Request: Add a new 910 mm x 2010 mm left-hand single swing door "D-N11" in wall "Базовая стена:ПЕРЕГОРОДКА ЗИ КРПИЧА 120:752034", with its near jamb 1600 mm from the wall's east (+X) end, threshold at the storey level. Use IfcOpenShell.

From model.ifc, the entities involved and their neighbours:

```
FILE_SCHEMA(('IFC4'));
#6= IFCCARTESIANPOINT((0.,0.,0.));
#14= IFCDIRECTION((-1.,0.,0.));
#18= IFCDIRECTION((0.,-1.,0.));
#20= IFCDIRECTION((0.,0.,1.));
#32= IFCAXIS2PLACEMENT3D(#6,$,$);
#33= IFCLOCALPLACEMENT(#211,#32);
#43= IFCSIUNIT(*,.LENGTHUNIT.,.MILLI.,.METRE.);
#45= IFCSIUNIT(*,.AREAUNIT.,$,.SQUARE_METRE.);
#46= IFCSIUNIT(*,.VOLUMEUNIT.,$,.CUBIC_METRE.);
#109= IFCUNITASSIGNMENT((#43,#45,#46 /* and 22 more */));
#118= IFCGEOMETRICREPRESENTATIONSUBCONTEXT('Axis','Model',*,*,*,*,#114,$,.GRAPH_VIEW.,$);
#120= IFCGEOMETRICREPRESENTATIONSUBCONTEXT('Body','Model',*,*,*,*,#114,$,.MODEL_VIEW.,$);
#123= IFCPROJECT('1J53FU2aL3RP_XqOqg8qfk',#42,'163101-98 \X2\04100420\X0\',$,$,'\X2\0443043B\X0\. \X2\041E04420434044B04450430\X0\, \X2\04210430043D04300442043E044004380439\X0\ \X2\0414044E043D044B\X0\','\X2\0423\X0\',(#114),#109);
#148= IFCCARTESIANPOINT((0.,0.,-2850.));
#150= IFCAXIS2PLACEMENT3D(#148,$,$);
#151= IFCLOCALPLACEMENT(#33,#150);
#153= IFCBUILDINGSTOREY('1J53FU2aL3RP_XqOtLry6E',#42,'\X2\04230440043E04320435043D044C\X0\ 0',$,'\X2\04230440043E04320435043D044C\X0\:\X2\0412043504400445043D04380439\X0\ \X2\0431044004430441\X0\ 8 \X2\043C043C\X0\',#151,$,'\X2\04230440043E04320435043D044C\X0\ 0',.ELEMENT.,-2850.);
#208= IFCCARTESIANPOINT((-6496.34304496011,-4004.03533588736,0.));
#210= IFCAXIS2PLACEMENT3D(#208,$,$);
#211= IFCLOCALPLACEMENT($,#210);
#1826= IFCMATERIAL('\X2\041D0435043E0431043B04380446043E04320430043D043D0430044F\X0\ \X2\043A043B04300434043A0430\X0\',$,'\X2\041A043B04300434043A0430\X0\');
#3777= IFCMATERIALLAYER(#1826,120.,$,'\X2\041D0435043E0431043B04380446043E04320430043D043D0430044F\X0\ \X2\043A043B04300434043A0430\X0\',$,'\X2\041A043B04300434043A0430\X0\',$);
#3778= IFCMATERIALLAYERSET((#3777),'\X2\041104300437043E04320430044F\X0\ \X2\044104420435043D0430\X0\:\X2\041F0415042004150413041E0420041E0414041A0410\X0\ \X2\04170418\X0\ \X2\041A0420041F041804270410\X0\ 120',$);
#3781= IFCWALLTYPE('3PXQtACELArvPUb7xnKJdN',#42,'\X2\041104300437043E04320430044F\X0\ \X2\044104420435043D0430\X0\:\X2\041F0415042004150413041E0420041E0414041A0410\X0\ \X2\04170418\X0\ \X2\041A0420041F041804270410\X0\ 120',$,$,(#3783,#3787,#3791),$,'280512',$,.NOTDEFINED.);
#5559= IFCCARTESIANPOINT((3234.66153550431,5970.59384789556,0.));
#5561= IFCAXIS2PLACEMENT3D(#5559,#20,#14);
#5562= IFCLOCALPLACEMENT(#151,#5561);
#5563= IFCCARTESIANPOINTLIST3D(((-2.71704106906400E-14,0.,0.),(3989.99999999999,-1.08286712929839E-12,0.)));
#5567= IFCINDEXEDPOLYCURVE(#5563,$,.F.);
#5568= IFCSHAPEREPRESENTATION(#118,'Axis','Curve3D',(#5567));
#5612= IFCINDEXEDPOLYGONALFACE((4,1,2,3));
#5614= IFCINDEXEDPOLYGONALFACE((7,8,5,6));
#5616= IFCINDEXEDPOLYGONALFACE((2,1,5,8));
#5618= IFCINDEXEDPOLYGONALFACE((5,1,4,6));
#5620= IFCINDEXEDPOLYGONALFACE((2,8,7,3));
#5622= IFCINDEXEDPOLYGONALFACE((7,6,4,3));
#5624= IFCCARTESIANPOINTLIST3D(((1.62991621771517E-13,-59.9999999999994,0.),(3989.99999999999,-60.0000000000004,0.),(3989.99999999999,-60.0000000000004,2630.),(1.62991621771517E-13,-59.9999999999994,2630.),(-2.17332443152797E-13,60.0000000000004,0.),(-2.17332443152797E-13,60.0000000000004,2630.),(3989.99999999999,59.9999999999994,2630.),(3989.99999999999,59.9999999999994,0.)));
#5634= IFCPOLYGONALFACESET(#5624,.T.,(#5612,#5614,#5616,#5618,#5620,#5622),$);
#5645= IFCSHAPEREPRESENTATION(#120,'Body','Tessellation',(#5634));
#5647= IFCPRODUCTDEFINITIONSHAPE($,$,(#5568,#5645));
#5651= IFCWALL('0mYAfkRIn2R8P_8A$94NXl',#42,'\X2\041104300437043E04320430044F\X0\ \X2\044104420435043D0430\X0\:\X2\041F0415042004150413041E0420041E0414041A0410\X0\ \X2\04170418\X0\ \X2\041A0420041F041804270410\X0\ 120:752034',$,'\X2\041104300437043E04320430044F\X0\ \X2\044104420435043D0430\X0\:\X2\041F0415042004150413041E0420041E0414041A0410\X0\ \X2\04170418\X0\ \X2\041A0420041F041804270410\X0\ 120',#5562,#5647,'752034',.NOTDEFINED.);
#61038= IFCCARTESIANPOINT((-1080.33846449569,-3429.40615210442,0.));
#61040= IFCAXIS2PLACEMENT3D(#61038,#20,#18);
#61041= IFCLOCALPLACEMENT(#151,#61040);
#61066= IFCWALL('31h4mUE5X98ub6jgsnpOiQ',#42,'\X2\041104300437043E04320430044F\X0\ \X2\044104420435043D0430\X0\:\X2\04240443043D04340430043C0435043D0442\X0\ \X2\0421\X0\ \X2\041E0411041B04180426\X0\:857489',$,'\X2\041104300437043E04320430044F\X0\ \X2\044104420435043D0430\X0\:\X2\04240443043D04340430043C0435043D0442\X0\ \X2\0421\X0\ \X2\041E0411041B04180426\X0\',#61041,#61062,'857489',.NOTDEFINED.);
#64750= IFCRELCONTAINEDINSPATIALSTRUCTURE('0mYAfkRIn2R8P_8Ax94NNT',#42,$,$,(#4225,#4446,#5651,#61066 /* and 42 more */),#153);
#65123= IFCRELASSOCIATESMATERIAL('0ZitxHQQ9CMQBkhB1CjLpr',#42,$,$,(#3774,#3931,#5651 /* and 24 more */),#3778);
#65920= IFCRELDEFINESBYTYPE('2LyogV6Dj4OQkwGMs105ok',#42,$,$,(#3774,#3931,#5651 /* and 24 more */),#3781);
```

```python
import numpy as np
import ifcopenshell
import ifcopenshell.api.feature
import ifcopenshell.api.geometry
import ifcopenshell.api.root
import ifcopenshell.api.spatial
import ifcopenshell.geom
import ifcopenshell.util.element
import ifcopenshell.util.placement
import ifcopenshell.util.representation
import ifcopenshell.util.shape
import ifcopenshell.util.unit

model = ifcopenshell.open("model.ifc")
unit_scale = ifcopenshell.util.unit.calculate_unit_scale(model)
settings = ifcopenshell.geom.settings()


def volume(element):
    """Net volume in cubic metres, openings subtracted."""
    shape = ifcopenshell.geom.create_shape(settings, element)
    return ifcopenshell.util.shape.get_volume(shape.geometry)


wall = model.by_id(5651)
storey = ifcopenshell.util.element.get_container(wall, ifc_class="IfcBuildingStorey")
context = ifcopenshell.util.representation.get_context(model, "Model", "Body", "MODEL_VIEW")
before = volume(wall)

width, height, from_end, sill = 0.91, 2.01, 1.6, 0.0  # metres

# The wall runs along its own X axis, and the end named is its -X end.
wall_shape = ifcopenshell.geom.create_shape(settings, wall)
x, y, z = ifcopenshell.util.shape.get_vertices(wall_shape.geometry).T
start = x.min() + from_end
face, thickness = float(y.min()), float(y.max() - y.min())
wall_matrix = ifcopenshell.util.placement.get_local_placement(wall.ObjectPlacement)
level = ifcopenshell.util.placement.get_local_placement(storey.ObjectPlacement)[2, 3]


def in_wall(x, y):
    """Placement at x, y metres in the wall's axes, at sill height."""
    matrix = wall_matrix.copy()
    matrix[:, 3] = wall_matrix @ np.array([x / unit_scale, y / unit_scale, 0.0, 1.0])
    matrix[2, 3] = level + sill / unit_scale
    return matrix


# Opening: a box that overshoots both wall faces by 50 mm.
opening = ifcopenshell.api.root.create_entity(model, ifc_class="IfcOpeningElement", predefined_type="OPENING")
box = ifcopenshell.api.geometry.add_wall_representation(
    model, context=context, length=width, height=height, thickness=thickness + 0.1
)
ifcopenshell.api.geometry.assign_representation(model, product=opening, representation=box)
ifcopenshell.api.geometry.edit_object_placement(model, product=opening, matrix=in_wall(start, face - 0.05), is_si=False)
ifcopenshell.api.feature.add_feature(model, feature=opening, element=wall)

door = ifcopenshell.api.root.create_entity(model, ifc_class="IfcDoor", name="D-N11", predefined_type="DOOR")
door.OverallWidth, door.OverallHeight = width / unit_scale, height / unit_scale
door.OperationType = "SINGLE_SWING_LEFT"
body = ifcopenshell.api.geometry.add_door_representation(
    model,
    context=context,
    overall_width=door.OverallWidth,
    overall_height=door.OverallHeight,
    operation_type="SINGLE_SWING_LEFT",
    lining_properties={"LiningDepth": thickness / unit_scale, "ThresholdDepth": thickness / unit_scale},
)
ifcopenshell.api.geometry.assign_representation(model, product=door, representation=body)
ifcopenshell.api.spatial.assign_container(model, products=[door], relating_structure=storey)
ifcopenshell.api.feature.add_filling(model, opening=opening, element=door)

# The lining spans the wall, so the door starts at the wall face.
ifcopenshell.api.geometry.edit_object_placement(model, product=door, matrix=in_wall(start, face), is_si=False)

after = volume(wall)

print(f"wall volume {before:.3f} -> {after:.3f} m3")

model.write("model_updated.ifc")
```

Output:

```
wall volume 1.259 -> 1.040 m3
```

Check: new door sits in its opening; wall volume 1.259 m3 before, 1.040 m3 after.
